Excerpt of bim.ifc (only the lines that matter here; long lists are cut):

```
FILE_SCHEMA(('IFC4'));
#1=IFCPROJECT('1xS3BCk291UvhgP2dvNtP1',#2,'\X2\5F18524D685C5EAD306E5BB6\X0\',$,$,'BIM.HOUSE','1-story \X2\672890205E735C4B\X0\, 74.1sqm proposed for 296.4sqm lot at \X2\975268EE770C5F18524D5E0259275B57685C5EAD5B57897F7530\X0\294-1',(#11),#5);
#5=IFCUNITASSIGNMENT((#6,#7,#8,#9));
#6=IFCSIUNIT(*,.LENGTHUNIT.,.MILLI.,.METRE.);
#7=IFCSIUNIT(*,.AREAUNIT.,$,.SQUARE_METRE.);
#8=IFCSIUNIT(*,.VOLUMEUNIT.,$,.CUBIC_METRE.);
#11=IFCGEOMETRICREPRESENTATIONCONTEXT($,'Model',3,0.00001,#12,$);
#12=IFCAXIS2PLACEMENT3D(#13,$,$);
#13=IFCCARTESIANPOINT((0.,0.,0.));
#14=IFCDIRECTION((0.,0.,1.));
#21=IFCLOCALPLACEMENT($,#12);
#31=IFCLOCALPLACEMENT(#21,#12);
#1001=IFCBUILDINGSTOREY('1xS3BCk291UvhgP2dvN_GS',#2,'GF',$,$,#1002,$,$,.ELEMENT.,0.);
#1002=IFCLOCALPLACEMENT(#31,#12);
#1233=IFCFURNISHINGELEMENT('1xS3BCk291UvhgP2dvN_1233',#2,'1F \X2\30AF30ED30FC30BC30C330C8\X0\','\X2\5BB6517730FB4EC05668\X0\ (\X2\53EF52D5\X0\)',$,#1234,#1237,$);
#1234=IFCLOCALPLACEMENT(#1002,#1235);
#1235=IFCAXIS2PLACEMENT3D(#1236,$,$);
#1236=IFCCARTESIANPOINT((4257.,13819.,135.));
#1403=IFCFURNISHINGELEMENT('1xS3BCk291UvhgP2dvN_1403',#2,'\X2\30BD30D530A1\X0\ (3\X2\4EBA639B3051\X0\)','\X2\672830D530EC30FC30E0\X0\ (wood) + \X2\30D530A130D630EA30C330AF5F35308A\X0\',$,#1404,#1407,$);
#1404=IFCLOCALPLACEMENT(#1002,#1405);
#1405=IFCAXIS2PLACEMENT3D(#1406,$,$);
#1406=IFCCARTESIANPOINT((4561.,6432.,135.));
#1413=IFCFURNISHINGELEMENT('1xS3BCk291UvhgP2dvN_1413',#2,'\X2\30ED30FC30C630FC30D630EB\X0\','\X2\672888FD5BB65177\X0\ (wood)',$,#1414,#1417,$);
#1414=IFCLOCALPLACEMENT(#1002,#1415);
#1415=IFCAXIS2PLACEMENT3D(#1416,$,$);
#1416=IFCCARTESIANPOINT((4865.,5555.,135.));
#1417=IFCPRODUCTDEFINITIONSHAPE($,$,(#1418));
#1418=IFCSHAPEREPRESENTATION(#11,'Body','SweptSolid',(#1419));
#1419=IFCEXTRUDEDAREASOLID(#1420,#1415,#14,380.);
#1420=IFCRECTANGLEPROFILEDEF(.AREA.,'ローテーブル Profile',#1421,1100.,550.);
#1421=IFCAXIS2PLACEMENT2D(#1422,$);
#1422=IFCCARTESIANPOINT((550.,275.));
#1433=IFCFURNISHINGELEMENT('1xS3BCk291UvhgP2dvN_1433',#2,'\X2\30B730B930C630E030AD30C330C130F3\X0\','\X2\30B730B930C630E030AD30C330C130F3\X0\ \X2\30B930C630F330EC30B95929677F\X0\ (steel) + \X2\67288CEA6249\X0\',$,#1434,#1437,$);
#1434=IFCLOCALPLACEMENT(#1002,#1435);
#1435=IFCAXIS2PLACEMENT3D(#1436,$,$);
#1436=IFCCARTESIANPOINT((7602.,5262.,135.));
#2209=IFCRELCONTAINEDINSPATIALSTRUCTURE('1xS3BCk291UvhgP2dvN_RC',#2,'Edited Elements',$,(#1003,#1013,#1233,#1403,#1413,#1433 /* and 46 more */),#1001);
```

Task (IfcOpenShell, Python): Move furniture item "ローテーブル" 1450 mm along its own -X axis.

```python
import ifcopenshell
import ifcopenshell.api.geometry
import ifcopenshell.util.placement
import ifcopenshell.util.unit

model = ifcopenshell.open("bim.ifc")
unit_scale = ifcopenshell.util.unit.calculate_unit_scale(model)

item = model.by_id(1413)
matrix = ifcopenshell.util.placement.get_local_placement(item.ObjectPlacement)
matrix[:3, 3] -= matrix[:3, 0] * 1.45 / unit_scale
ifcopenshell.api.geometry.edit_object_placement(model, product=item, matrix=matrix, is_si=False)

print(ifcopenshell.util.placement.get_local_placement(item.ObjectPlacement).round(3) + 0.0)

model.write("bim-out.ifc")
```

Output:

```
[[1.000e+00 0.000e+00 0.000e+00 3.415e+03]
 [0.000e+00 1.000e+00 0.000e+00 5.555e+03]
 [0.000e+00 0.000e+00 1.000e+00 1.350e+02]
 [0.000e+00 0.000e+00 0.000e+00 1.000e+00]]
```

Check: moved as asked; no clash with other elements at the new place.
